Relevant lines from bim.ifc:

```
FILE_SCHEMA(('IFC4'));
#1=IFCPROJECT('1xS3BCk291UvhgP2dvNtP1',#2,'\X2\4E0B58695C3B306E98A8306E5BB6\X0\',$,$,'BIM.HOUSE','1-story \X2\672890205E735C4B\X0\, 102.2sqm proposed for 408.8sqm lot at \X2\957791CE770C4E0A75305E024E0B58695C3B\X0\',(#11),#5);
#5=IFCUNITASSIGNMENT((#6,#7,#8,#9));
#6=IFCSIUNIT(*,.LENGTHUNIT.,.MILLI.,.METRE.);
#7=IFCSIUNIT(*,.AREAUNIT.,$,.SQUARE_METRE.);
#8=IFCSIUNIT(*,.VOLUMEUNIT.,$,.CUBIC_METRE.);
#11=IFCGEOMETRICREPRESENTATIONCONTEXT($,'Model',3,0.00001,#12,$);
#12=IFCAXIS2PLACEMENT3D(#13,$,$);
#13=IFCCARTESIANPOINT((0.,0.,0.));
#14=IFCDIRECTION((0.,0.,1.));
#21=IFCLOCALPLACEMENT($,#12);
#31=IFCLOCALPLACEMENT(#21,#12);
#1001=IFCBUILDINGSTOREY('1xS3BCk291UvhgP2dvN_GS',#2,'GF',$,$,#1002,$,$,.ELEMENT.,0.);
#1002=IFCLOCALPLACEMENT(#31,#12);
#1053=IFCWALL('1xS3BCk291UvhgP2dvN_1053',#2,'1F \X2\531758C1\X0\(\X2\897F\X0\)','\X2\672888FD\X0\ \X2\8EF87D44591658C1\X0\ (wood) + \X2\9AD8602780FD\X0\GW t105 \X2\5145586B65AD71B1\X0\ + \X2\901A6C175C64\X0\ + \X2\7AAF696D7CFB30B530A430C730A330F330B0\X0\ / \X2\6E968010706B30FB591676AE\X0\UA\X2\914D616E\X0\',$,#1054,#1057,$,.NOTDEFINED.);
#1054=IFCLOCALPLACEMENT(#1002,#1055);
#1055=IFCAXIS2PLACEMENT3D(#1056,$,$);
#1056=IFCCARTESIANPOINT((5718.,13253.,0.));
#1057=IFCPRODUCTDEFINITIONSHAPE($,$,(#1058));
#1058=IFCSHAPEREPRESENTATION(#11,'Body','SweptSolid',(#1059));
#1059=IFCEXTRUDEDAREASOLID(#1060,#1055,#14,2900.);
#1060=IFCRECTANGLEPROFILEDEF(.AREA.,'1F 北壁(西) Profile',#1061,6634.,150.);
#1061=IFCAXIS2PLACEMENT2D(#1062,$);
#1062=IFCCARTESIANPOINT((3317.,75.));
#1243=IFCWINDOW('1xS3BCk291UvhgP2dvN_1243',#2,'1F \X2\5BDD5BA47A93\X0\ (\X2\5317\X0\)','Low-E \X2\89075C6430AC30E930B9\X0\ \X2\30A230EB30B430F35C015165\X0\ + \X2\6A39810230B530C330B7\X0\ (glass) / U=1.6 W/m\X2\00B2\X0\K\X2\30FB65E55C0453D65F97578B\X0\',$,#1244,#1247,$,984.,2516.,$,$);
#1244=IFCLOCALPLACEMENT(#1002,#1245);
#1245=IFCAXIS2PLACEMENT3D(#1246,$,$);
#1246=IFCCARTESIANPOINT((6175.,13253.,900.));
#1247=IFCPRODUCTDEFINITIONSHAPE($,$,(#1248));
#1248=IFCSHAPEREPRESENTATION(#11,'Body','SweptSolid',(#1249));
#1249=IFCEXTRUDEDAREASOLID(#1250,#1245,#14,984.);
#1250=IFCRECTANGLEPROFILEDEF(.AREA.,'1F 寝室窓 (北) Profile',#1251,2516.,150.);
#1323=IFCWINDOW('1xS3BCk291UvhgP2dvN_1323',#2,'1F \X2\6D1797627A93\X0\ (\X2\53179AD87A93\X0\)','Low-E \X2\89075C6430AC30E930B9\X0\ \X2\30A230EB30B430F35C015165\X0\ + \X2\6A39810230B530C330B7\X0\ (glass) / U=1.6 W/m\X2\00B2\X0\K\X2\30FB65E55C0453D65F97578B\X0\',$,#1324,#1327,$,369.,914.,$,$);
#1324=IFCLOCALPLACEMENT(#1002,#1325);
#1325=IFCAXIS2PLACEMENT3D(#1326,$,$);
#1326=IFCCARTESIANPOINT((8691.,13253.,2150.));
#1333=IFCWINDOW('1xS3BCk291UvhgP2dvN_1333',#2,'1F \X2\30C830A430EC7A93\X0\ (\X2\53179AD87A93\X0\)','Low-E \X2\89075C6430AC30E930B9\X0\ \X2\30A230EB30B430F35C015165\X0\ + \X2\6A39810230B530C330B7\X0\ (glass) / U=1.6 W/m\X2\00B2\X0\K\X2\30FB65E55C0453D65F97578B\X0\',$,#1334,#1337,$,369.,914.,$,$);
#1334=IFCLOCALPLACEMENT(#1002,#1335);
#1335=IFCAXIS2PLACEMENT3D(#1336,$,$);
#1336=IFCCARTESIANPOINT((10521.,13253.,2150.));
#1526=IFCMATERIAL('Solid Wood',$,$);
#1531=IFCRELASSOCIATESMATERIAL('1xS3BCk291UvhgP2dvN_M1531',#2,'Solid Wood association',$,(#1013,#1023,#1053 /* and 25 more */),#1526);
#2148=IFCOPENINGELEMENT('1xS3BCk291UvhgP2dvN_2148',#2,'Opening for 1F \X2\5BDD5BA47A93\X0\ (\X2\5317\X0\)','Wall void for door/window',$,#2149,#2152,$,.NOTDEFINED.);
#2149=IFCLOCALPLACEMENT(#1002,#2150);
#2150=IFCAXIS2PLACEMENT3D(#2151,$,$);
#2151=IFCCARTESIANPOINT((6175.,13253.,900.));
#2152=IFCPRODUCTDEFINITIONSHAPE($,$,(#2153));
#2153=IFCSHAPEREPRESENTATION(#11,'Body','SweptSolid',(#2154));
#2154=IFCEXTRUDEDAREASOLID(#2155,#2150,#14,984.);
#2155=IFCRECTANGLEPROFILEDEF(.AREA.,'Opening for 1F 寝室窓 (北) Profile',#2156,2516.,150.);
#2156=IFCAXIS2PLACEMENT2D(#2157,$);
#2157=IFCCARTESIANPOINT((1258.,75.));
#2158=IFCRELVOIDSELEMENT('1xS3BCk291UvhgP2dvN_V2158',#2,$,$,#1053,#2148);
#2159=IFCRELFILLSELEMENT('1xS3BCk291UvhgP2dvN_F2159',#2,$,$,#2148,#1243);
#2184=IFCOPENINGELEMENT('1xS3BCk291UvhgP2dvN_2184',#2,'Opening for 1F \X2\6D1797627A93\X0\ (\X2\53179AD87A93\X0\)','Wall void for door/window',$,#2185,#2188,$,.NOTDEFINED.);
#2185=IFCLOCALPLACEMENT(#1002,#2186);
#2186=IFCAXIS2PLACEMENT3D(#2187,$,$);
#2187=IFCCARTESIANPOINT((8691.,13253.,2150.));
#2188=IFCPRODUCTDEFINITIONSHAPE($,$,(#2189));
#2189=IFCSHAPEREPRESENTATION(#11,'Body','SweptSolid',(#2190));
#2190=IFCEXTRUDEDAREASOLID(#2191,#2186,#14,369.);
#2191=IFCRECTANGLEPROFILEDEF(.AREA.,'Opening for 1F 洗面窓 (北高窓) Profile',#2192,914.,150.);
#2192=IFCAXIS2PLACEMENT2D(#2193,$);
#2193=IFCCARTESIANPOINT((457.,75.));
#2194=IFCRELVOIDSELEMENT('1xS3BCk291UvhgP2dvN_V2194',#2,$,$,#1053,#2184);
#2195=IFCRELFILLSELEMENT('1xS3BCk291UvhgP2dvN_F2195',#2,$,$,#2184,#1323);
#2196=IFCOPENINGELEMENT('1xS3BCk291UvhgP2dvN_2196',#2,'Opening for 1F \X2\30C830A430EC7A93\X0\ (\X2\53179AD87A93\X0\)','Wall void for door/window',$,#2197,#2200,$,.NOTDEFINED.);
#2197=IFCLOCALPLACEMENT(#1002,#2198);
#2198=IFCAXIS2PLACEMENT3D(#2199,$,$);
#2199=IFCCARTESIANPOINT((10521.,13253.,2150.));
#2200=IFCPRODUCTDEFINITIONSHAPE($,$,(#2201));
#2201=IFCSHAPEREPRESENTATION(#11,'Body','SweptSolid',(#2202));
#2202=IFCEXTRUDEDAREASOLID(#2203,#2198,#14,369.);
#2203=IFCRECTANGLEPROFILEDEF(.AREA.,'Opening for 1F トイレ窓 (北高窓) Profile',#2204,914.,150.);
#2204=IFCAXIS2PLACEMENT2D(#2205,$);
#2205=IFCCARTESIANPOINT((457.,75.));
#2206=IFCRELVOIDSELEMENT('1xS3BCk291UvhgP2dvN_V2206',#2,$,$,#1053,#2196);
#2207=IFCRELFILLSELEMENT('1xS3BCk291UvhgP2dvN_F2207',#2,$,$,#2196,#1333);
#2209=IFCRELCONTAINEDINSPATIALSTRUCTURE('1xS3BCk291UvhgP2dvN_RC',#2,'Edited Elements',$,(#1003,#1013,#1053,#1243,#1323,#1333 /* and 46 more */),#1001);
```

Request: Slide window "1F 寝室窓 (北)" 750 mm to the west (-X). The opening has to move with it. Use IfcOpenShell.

```python
import ifcopenshell
import ifcopenshell.api.geometry
import ifcopenshell.util.placement

model = ifcopenshell.open("bim.ifc")

window = model.by_guid("1xS3BCk291UvhgP2dvN_1243")
opening = window.FillsVoids[0].RelatingOpeningElement
wall = opening.VoidsElements[0].RelatingBuildingElement

wall_matrix = ifcopenshell.util.placement.get_local_placement(wall.ObjectPlacement)
shift = wall_matrix[:3, 0] * -750.0
before = ifcopenshell.util.placement.get_local_placement(window.ObjectPlacement)[:3, 3].copy()

# The window is not placed relative to its opening, so move both.
for product in (opening, window):
    matrix = ifcopenshell.util.placement.get_local_placement(product.ObjectPlacement)
    matrix[:3, 3] += shift
    ifcopenshell.api.geometry.edit_object_placement(model, product=product, matrix=matrix, is_si=False)

after = ifcopenshell.util.placement.get_local_placement(window.ObjectPlacement)[:3, 3]
print("window moved by", (after - before).round(3) + 0.0)

model.write("bim_rev.ifc")
```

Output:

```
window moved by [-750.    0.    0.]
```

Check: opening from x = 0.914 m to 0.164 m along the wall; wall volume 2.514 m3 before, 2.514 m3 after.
